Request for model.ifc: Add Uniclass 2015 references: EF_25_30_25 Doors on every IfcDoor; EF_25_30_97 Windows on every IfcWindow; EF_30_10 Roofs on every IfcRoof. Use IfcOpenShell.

First a look at what the model holds.

```python
import ifcopenshell

model = ifcopenshell.open("model.ifc")
print(model.schema)
print("classifications:", [c.Name for c in model.by_type("IfcClassification")])
for ifc_class in ("IfcDoor", "IfcRoof", "IfcStair", "IfcWall", "IfcWindow"):
    print(ifc_class, len(model.by_type(ifc_class)))
```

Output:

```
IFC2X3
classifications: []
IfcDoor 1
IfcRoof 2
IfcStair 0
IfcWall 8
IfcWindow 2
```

```python
import ifcopenshell
import ifcopenshell.api.classification

model = ifcopenshell.open("model.ifc")

# IFC2X3 requires Source and Edition and has no link from the project to the system.
system = model.create_entity("IfcClassification", Source="NBS", Edition="2015", Name="Uniclass 2015")

codes = {
    "IfcDoor": ("EF_25_30_25", "Doors"),
    "IfcWindow": ("EF_25_30_97", "Windows"),
    "IfcRoof": ("EF_30_10", "Roofs"),
}
for ifc_class, (code, name) in codes.items():
    products = model.by_type(ifc_class)
    ifcopenshell.api.classification.add_reference(
        model, products=products, classification=system, identification=code, name=name
    )
    print(code, len(products))

model.write("model_updated.ifc")
```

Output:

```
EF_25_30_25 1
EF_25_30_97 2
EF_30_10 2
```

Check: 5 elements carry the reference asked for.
